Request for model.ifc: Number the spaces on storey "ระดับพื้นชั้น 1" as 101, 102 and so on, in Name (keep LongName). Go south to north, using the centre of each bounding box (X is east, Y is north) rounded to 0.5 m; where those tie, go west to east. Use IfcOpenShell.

First a look at what the model holds.

```python
import ifcopenshell
import ifcopenshell.util.element
import ifcopenshell.util.placement

model = ifcopenshell.open("model.ifc")
print(model.schema)
storey = next(s for s in model.by_type("IfcBuildingStorey") if s.Name == "ระดับพื้นชั้น 1")
spaces = [e for e in ifcopenshell.util.element.get_decomposition(storey) if e.is_a("IfcSpace")]
for e in sorted(spaces, key=lambda e: e.id()):
    origin = ifcopenshell.util.placement.get_local_placement(e.ObjectPlacement)[:3, 3]
    print(e.id(), e.Name, e.LongName, origin.round(2) + 0.0, sep=" | ")
```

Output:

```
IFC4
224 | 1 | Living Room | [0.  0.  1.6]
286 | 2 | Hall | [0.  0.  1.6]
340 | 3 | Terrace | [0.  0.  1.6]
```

```python
import ifcopenshell
import ifcopenshell.geom
import ifcopenshell.util.element
import ifcopenshell.util.shape

model = ifcopenshell.open("model.ifc")
settings = ifcopenshell.geom.settings()
settings.set("use-world-coords", True)


def centre(element):
    shape = ifcopenshell.geom.create_shape(settings, element)
    return ifcopenshell.util.shape.get_bbox_centroid(shape.geometry)


storey = next(s for s in model.by_type("IfcBuildingStorey") if s.Name == "ระดับพื้นชั้น 1")
spaces = [e for e in ifcopenshell.util.element.get_decomposition(storey) if e.is_a("IfcSpace")]

# Insertion points can sit at a corner or the storey origin, so sort by the geometry (in metres).
centres = {e: centre(e) for e in spaces}
spaces.sort(key=lambda e: (round(centres[e][1] / 0.5), centres[e][0]))

for i, e in enumerate(spaces, start=1):
    number = f"1{i:02d}"
    e.Name = number
    print(e.id(), number)

model.write("model_v2.ifc")
```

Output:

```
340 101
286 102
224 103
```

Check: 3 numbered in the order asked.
